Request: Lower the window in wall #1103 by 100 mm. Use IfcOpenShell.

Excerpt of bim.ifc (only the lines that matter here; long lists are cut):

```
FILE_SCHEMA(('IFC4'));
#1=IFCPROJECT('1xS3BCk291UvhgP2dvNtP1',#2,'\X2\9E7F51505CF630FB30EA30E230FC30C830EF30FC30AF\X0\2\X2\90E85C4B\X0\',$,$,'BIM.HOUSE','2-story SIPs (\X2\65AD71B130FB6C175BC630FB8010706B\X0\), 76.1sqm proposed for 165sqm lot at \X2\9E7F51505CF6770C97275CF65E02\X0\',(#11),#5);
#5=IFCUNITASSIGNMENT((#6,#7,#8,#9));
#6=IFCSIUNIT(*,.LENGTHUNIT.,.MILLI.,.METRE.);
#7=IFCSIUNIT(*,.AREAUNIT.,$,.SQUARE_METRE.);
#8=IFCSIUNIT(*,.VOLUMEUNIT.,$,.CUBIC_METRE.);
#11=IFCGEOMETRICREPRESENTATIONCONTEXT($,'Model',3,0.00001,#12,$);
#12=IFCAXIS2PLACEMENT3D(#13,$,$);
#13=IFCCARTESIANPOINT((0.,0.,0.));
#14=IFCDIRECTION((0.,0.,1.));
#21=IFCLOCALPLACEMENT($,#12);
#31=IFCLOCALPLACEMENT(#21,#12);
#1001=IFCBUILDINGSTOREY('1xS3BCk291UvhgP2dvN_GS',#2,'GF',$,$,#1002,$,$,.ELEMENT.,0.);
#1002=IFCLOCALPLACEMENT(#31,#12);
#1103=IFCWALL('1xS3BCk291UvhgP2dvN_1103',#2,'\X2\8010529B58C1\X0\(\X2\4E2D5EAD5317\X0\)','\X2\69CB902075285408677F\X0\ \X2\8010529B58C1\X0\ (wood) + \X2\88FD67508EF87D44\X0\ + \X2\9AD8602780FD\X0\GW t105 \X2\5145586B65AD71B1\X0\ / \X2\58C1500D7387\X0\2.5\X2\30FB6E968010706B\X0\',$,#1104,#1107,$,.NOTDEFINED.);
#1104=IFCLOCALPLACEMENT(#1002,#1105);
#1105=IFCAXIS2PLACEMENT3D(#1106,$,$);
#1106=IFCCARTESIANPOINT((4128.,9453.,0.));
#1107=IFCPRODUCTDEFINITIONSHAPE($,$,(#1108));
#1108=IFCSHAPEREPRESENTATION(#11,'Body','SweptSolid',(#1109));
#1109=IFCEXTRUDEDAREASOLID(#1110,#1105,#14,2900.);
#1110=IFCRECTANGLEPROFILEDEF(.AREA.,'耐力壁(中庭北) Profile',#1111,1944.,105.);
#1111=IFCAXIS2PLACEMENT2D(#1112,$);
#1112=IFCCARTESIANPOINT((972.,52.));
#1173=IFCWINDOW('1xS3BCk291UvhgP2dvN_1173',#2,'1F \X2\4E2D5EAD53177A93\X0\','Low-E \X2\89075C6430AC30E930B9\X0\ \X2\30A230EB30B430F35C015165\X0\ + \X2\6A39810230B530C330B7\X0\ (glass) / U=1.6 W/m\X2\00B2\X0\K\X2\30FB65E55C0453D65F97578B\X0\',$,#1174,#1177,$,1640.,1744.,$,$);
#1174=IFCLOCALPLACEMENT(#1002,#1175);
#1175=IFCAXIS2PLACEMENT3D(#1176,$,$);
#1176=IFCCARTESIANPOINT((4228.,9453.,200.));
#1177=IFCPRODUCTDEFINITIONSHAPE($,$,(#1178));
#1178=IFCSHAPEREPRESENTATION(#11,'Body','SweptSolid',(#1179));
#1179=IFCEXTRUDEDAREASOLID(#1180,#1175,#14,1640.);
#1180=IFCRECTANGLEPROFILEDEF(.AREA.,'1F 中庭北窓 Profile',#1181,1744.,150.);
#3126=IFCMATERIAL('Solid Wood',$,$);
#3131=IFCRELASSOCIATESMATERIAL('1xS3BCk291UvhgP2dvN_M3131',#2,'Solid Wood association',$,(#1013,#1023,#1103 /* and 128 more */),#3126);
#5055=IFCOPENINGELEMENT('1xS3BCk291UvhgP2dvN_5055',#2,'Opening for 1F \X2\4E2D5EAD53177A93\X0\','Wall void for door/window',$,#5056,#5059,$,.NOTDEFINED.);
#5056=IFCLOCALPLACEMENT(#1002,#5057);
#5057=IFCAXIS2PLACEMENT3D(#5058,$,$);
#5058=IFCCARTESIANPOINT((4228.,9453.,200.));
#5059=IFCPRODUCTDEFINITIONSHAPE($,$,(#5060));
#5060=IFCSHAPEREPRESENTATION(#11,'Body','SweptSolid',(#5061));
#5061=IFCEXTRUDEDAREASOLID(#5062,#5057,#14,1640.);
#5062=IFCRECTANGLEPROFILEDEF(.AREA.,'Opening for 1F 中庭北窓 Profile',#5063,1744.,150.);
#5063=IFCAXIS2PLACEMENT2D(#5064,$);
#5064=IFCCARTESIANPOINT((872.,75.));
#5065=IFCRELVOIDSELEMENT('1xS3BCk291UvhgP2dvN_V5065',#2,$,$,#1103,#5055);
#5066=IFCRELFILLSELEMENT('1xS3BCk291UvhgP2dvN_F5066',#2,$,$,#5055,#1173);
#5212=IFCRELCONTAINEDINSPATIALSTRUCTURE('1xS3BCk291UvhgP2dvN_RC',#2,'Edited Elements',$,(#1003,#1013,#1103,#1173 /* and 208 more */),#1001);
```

```python
import numpy as np
import ifcopenshell
import ifcopenshell.api.geometry
import ifcopenshell.util.placement
import ifcopenshell.util.unit

model = ifcopenshell.open("bim.ifc")
unit_scale = ifcopenshell.util.unit.calculate_unit_scale(model)

window = model.by_guid("1xS3BCk291UvhgP2dvN_1173")
opening = window.FillsVoids[0].RelatingOpeningElement
dz = -0.1 / unit_scale

shift = np.array([0.0, 0.0, dz])
# The window is not placed relative to its opening, so move both.
for product in (opening, window):
    matrix = ifcopenshell.util.placement.get_local_placement(product.ObjectPlacement)
    matrix[:3, 3] += shift
    ifcopenshell.api.geometry.edit_object_placement(model, product=product, matrix=matrix, is_si=False)

print(f"moved by {dz * unit_scale:+.3f} m")

model.write("bim_v2.ifc")
```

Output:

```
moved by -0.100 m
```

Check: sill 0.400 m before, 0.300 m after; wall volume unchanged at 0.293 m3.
